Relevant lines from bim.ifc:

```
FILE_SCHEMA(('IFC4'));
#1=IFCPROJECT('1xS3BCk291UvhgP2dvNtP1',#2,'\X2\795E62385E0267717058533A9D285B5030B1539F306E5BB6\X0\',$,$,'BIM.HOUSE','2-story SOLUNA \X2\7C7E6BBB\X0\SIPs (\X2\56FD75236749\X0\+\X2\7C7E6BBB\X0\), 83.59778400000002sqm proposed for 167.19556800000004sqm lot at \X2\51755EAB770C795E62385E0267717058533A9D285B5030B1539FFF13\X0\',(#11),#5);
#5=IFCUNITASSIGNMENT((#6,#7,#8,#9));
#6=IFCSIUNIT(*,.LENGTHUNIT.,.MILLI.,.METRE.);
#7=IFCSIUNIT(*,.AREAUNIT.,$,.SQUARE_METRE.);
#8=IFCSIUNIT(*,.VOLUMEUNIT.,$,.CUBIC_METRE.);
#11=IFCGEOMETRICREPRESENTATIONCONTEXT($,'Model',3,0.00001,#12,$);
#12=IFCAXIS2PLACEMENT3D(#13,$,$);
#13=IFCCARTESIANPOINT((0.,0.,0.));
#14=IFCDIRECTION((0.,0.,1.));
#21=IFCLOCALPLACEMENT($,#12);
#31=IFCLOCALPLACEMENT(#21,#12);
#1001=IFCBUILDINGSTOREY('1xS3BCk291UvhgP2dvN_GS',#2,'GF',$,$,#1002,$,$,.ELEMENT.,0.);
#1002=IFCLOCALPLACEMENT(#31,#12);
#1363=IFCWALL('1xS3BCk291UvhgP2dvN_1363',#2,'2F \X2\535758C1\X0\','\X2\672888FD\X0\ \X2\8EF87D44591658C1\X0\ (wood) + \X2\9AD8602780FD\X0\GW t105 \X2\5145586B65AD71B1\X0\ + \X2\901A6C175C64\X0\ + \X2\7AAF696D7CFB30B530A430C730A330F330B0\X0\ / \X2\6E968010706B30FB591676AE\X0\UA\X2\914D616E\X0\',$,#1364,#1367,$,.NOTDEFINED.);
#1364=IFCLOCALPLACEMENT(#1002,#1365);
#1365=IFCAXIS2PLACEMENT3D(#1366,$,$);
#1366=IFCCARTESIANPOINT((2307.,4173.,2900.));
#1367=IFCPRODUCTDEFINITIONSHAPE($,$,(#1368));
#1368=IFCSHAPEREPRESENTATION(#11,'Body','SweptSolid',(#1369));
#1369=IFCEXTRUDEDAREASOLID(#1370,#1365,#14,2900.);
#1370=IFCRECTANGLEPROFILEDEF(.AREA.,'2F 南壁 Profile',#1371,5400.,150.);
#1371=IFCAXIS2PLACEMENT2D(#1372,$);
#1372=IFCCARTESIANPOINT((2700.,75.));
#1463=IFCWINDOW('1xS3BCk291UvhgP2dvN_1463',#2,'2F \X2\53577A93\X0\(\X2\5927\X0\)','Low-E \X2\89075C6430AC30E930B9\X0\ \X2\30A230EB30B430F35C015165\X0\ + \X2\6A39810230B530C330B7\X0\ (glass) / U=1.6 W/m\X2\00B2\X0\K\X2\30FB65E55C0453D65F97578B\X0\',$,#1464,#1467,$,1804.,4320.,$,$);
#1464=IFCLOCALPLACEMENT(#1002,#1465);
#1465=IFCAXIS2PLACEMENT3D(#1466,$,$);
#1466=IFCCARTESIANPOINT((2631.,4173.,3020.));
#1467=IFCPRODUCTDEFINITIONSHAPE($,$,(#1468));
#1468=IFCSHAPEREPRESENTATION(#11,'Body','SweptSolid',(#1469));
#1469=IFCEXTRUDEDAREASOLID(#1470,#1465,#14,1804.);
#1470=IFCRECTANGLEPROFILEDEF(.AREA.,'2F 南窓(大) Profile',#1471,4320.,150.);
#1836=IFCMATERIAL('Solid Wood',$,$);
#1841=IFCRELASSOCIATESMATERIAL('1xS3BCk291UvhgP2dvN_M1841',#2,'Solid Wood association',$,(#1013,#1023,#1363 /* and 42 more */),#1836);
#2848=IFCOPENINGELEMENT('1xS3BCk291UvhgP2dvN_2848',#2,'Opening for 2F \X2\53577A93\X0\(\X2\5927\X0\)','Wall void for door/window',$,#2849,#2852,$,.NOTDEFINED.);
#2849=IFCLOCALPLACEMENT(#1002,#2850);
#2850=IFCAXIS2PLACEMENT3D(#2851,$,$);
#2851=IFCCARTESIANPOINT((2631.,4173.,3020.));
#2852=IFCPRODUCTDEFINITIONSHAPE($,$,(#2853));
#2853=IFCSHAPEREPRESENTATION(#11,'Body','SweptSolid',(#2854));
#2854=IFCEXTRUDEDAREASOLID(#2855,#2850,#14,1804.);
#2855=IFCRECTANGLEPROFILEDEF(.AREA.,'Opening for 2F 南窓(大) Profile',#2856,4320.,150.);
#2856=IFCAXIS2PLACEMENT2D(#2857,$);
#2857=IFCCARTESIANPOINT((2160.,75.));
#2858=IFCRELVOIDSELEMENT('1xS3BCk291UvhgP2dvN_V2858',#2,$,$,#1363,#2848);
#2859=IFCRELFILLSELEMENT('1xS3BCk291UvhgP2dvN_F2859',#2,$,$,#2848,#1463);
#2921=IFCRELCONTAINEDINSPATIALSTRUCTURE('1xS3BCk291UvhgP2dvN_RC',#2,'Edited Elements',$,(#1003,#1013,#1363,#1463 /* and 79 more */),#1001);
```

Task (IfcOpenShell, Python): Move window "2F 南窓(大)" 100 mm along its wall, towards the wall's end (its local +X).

```python
import ifcopenshell
import ifcopenshell.api.geometry
import ifcopenshell.util.placement

model = ifcopenshell.open("bim.ifc")

window = model.by_id(1463)
opening = window.FillsVoids[0].RelatingOpeningElement
wall = opening.VoidsElements[0].RelatingBuildingElement

wall_matrix = ifcopenshell.util.placement.get_local_placement(wall.ObjectPlacement)
shift = wall_matrix[:3, 0] * 100.0
before = ifcopenshell.util.placement.get_local_placement(window.ObjectPlacement)[:3, 3].copy()

# The window is not placed relative to its opening, so move both.
for product in (opening, window):
    matrix = ifcopenshell.util.placement.get_local_placement(product.ObjectPlacement)
    matrix[:3, 3] += shift
    ifcopenshell.api.geometry.edit_object_placement(model, product=product, matrix=matrix, is_si=False)

after = ifcopenshell.util.placement.get_local_placement(window.ObjectPlacement)[:3, 3]
print("window moved by", (after - before).round(3) + 0.0)

model.write("bim_edited.ifc")
```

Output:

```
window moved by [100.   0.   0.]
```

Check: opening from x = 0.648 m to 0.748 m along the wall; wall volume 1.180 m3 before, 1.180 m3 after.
